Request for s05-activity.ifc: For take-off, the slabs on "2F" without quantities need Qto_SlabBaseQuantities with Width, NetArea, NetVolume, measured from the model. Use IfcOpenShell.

First a look at what the model holds.

```python
import ifcopenshell
import ifcopenshell.util.element
import ifcopenshell.util.unit

model = ifcopenshell.open("s05-activity.ifc")
print(model.schema)
for unit_type in ("LENGTHUNIT", "AREAUNIT", "VOLUMEUNIT"):
    print(unit_type, ifcopenshell.util.unit.calculate_unit_scale(model, unit_type))
storey = next(s for s in model.by_type("IfcBuildingStorey") if s.Name == "2F")
slabs = [e for e in ifcopenshell.util.element.get_decomposition(storey) if e.is_a("IfcSlab")]
for e in sorted(slabs, key=lambda e: e.id()):
    print(e.id(), e.is_a(), e.Name, list(ifcopenshell.util.element.get_psets(e, qtos_only=True)), sep=" | ")
```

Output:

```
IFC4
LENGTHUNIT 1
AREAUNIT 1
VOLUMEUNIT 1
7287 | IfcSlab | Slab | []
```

```python
import ifcopenshell
import ifcopenshell.api.pset
import ifcopenshell.geom
import ifcopenshell.util.element
import ifcopenshell.util.shape
import ifcopenshell.util.unit

model = ifcopenshell.open("s05-activity.ifc")
unit_scale = ifcopenshell.util.unit.calculate_unit_scale(model)
area_scale = ifcopenshell.util.unit.calculate_unit_scale(model, "AREAUNIT")
volume_scale = ifcopenshell.util.unit.calculate_unit_scale(model, "VOLUMEUNIT")
settings = ifcopenshell.geom.settings()

storey = next(s for s in model.by_type("IfcBuildingStorey") if s.Name == "2F")
slabs = [e for e in ifcopenshell.util.element.get_decomposition(storey) if e.is_a("IfcSlab")]

for e in sorted(slabs, key=lambda e: e.id()):
    if ifcopenshell.util.element.get_psets(e, qtos_only=True, should_inherit=False):
        continue
    # Geometry comes back in metres, in the element's own axes.
    shape = ifcopenshell.geom.create_shape(settings, e)
    values = {
        "Width": ifcopenshell.util.shape.get_z(shape.geometry) / unit_scale,
        "NetArea": ifcopenshell.util.shape.get_footprint_area(shape.geometry) / area_scale,
        "NetVolume": ifcopenshell.util.shape.get_volume(shape.geometry) / volume_scale,
    }
    qto = ifcopenshell.api.pset.add_qto(model, product=e, name="Qto_SlabBaseQuantities")
    ifcopenshell.api.pset.edit_qto(model, qto=qto, properties=values)
    print(e.id(), {k: round(v, 3) for k, v in values.items()})

model.write("s05-activity_updated.ifc")
```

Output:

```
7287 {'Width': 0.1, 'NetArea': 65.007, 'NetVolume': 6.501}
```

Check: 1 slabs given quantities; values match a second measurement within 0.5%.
